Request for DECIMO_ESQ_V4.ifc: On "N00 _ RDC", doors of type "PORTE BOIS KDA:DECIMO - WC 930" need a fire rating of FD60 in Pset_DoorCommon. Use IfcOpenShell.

First a look at what the model holds.

```python
import ifcopenshell
import ifcopenshell.util.element

model = ifcopenshell.open("DECIMO_ESQ_V4.ifc")
print(model.schema)
storey = next(s for s in model.by_type("IfcBuildingStorey") if s.Name == "N00 _ RDC")
doors = [e for e in ifcopenshell.util.element.get_decomposition(storey) if e.is_a("IfcDoor")]
seen = {}
for e in doors:
    element_type = ifcopenshell.util.element.get_type(e)
    key = (element_type.Name if element_type != e and element_type else None, ifcopenshell.util.element.get_pset(e, "Pset_DoorCommon", "FireRating"))
    seen[key] = seen.get(key, 0) + 1
for (name, value), count in sorted(seen.items(), key=str):
    print(count, "x", name, "|", value)
```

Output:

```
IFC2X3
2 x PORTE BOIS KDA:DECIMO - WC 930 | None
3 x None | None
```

```python
import ifcopenshell
import ifcopenshell.api.pset
import ifcopenshell.util.element

model = ifcopenshell.open("DECIMO_ESQ_V4.ifc")

storey = next(s for s in model.by_type("IfcBuildingStorey") if s.Name == "N00 _ RDC")
doors = [e for e in ifcopenshell.util.element.get_decomposition(storey) if e.is_a("IfcDoor")]

count = 0
for e in doors:
    element_type = ifcopenshell.util.element.get_type(e)
    if element_type in (None, e) or element_type.Name != "PORTE BOIS KDA:DECIMO - WC 930":
        continue
    # add_pset returns the element's existing set when there is one.
    pset = ifcopenshell.api.pset.add_pset(model, product=e, name="Pset_DoorCommon")
    ifcopenshell.api.pset.edit_pset(model, pset=pset, properties={"FireRating": "FD60"})
    count += 1

print(count, "doors updated")

model.write("DECIMO_ESQ_V4_edited.ifc")
```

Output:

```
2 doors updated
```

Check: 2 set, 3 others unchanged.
